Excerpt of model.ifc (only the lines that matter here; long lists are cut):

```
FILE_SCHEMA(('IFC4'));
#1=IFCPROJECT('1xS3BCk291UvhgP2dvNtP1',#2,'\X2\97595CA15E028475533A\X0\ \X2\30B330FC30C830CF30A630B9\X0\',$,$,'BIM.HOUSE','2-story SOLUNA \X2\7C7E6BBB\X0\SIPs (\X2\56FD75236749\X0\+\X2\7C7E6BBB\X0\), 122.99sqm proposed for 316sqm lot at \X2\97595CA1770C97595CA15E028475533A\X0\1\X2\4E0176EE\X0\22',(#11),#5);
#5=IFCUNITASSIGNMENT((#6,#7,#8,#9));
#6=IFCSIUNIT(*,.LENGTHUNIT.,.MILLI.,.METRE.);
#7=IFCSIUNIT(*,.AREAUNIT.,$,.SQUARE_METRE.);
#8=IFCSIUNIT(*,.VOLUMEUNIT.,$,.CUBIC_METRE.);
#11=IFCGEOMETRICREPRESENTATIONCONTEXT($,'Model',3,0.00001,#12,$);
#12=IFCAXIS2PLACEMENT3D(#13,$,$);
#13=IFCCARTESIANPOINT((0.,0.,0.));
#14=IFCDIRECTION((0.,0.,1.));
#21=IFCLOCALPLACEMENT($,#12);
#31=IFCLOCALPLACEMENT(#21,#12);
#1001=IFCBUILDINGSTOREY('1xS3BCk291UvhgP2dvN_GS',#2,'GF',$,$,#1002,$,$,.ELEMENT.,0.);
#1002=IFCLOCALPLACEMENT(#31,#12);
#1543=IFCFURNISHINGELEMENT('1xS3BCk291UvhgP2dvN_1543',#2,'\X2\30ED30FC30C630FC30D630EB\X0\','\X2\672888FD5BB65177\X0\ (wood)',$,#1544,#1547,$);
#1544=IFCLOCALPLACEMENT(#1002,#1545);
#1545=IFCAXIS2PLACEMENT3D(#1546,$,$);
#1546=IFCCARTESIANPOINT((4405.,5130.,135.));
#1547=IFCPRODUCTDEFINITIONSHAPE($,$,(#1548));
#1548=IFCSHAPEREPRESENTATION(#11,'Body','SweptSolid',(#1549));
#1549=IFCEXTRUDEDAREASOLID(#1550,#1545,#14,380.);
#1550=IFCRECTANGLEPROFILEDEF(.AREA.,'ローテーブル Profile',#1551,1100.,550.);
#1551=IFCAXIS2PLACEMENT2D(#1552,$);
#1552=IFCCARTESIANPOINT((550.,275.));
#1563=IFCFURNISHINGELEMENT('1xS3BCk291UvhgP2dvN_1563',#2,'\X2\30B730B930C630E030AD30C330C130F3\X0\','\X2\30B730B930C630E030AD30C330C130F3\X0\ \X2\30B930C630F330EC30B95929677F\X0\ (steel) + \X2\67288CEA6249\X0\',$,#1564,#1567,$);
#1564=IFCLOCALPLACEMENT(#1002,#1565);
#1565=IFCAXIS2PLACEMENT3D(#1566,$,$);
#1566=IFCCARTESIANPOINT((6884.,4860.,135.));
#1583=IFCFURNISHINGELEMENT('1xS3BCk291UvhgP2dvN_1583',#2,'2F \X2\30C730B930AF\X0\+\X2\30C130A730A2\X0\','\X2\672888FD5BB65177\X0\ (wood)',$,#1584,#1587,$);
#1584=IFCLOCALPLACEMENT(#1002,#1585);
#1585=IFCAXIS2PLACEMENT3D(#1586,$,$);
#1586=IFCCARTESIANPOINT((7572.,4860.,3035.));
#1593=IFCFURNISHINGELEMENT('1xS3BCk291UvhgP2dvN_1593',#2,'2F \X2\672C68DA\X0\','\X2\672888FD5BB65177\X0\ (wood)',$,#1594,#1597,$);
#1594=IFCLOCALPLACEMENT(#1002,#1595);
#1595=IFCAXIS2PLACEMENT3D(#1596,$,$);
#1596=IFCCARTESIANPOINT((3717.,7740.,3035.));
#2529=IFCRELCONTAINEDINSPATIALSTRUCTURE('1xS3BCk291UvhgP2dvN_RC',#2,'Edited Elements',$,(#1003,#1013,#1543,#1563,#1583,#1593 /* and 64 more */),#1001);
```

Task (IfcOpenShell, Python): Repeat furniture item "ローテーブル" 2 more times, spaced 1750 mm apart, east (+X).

```python
import numpy as np
import ifcopenshell
import ifcopenshell.api.geometry
import ifcopenshell.api.root
import ifcopenshell.util.element
import ifcopenshell.util.placement
import ifcopenshell.util.unit

model = ifcopenshell.open("model.ifc")
unit_scale = ifcopenshell.util.unit.calculate_unit_scale(model)


def reuse_history(source, copy):
    """copy_class also copies each property set's owner history, people and application; keep the originals."""
    for rel in copy.IsDefinedBy:
        if rel.is_a("IfcRelDefinesByProperties") and (history := rel.RelatingPropertyDefinition.OwnerHistory):
            rel.RelatingPropertyDefinition.OwnerHistory = source.OwnerHistory
            ifcopenshell.util.element.remove_deep2(model, history)


source = model.by_id(1543)
base = ifcopenshell.util.placement.get_local_placement(source.ObjectPlacement)
step = np.array([1.0, 0.0, 0.0]) * 1.75 / unit_scale

for i in range(1, 3):
    copy = ifcopenshell.api.root.copy_class(model, product=source)
    copy.Representation = ifcopenshell.util.element.copy_deep(
        model, source.Representation, exclude=["IfcGeometricRepresentationContext", "IfcRepresentationMap"]
    )
    reuse_history(source, copy)
    matrix = base.copy()
    matrix[:3, 3] += i * step
    print("added at", matrix[:3, 3].round(3) + 0.0)
    ifcopenshell.api.geometry.edit_object_placement(model, product=copy, matrix=matrix, is_si=False)

model.write("model_edited.ifc")
```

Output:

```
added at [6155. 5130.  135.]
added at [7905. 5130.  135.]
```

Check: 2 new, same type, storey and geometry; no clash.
